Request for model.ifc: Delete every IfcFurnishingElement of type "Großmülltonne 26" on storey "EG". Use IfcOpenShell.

First a look at what the model holds.

```python
import ifcopenshell
import ifcopenshell.util.element

model = ifcopenshell.open("model.ifc")
print(model.schema)
storey = next(s for s in model.by_type("IfcBuildingStorey") if s.Name == "EG")
furniture = [e for e in ifcopenshell.util.element.get_decomposition(storey) if e.is_a("IfcFurnishingElement")]
seen = {}
for e in furniture:
    element_type = ifcopenshell.util.element.get_type(e)
    name = element_type.Name if element_type not in (None, e) else None
    seen[name] = seen.get(name, 0) + 1
for name, count in sorted(seen.items(), key=str):
    print(count, "x", name)
```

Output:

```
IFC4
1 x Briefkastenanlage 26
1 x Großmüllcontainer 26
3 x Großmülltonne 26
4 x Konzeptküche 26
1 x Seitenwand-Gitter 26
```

```python
import ifcopenshell
import ifcopenshell.api.root
import ifcopenshell.util.element

model = ifcopenshell.open("model.ifc")

storey = next(s for s in model.by_type("IfcBuildingStorey") if s.Name == "EG")
furniture = [e for e in ifcopenshell.util.element.get_decomposition(storey) if e.is_a("IfcFurnishingElement")]
targets = [e for e in furniture if (t := ifcopenshell.util.element.get_type(e)) not in (None, e) and t.Name == "Großmülltonne 26"]

for e in targets:
    ifcopenshell.api.root.remove_product(model, product=e)
print(len(targets), "removed")

model.write("model-out.ifc")
```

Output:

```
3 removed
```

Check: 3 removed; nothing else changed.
